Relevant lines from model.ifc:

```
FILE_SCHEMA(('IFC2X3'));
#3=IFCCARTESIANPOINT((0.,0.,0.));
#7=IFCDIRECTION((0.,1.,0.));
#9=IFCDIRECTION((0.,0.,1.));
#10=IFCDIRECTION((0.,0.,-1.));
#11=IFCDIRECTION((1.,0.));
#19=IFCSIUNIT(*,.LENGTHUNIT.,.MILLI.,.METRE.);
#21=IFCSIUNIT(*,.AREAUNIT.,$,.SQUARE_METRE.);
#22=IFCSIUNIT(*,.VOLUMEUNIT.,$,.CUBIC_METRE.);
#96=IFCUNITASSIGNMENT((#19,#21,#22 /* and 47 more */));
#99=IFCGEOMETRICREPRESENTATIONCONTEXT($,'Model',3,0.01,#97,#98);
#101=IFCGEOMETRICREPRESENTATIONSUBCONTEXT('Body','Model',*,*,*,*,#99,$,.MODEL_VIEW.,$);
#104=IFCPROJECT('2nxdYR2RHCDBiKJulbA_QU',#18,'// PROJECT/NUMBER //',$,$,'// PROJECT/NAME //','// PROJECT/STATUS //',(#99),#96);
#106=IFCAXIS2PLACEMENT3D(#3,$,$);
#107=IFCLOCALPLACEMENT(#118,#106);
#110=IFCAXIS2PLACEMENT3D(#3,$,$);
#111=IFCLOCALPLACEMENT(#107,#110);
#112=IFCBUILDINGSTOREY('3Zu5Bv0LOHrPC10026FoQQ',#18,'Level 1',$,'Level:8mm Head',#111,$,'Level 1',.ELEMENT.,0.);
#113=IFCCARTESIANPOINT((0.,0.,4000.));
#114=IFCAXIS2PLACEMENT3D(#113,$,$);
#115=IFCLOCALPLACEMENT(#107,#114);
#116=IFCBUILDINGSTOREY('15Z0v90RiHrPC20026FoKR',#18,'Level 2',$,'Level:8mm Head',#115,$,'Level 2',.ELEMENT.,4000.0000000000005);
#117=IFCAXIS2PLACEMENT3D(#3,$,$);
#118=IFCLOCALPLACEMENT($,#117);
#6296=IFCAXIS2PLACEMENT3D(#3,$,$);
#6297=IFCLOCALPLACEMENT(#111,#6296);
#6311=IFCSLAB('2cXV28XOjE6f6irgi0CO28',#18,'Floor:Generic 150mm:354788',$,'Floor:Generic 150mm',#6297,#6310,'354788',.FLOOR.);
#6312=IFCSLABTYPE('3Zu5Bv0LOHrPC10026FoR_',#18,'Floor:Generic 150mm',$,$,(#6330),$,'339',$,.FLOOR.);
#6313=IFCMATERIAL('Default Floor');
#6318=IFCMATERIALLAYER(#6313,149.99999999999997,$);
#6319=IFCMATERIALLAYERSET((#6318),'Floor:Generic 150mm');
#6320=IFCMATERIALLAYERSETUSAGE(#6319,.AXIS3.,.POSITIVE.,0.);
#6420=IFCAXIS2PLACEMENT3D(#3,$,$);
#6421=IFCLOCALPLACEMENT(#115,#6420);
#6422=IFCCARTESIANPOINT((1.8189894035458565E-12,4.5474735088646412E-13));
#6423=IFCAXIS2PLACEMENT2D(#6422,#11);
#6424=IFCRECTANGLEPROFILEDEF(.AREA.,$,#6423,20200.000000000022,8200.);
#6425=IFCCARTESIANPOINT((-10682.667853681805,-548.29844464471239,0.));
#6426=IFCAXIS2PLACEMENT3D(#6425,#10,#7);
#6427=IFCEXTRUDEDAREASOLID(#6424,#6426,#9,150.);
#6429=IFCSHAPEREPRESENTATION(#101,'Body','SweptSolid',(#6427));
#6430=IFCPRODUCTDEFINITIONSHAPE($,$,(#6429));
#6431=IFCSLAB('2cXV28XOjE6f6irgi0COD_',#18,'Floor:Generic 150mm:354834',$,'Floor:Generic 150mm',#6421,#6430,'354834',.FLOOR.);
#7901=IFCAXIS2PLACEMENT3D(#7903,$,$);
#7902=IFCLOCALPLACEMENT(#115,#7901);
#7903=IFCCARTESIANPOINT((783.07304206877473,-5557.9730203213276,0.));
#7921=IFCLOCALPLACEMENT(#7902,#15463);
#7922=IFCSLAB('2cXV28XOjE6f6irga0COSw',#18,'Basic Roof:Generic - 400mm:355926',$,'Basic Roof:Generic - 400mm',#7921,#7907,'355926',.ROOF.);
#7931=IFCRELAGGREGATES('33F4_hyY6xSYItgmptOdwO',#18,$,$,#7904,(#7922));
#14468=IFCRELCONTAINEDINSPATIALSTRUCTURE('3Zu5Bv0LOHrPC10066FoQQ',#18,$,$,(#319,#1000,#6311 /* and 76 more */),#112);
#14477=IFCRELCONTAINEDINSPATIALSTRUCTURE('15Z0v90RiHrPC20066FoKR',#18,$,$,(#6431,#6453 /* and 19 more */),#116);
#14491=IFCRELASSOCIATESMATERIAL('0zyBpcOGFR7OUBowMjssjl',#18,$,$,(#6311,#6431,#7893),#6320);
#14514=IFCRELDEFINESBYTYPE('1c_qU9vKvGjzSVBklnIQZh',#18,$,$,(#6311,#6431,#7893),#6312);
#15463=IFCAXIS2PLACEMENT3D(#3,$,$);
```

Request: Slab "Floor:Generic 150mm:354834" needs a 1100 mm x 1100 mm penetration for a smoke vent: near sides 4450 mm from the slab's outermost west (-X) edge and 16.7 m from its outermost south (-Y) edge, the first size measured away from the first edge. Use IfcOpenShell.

```python
import numpy as np
import ifcopenshell
import ifcopenshell.api.feature
import ifcopenshell.api.geometry
import ifcopenshell.api.root
import ifcopenshell.geom
import ifcopenshell.util.placement
import ifcopenshell.util.representation
import ifcopenshell.util.shape
import ifcopenshell.util.unit

model = ifcopenshell.open("model.ifc")
unit_scale = ifcopenshell.util.unit.calculate_unit_scale(model)
settings = ifcopenshell.geom.settings()


def volume(element):
    """Net volume in cubic metres, openings subtracted."""
    shape = ifcopenshell.geom.create_shape(settings, element)
    return ifcopenshell.util.shape.get_volume(shape.geometry)


slab = model.by_id(6431)
before = volume(slab)

# Extent in the slab's own axes, in metres. The edges named are its -X and -Y sides.
slab_shape = ifcopenshell.geom.create_shape(settings, slab)
vertices = ifcopenshell.util.shape.get_vertices(slab_shape.geometry)
x_min, y_min, bottom = vertices.min(axis=0)
top = vertices[:, 2].max()

opening = ifcopenshell.api.root.create_entity(model, ifc_class="IfcOpeningElement", name="Smoke vent opening")
context = ifcopenshell.util.representation.get_context(model, "Model", "Body", "MODEL_VIEW")
width, depth = 1.1, 1.1
outline = [(0.0, 0.0), (width, 0.0), (width, depth), (0.0, depth), (0.0, 0.0)]
# Overshoot both faces by 50 mm so the cut is clean.
shape = ifcopenshell.api.geometry.add_slab_representation(
    model, context=context, depth=top - bottom + 0.1, polyline=outline
)
ifcopenshell.api.geometry.assign_representation(model, product=opening, representation=shape)

matrix = ifcopenshell.util.placement.get_local_placement(slab.ObjectPlacement)
matrix[:, 3] = matrix @ np.append(np.array([x_min + 4.45, y_min + 16.7, bottom - 0.05]) / unit_scale, 1.0)
ifcopenshell.api.geometry.edit_object_placement(model, product=opening, matrix=matrix, is_si=False)
ifcopenshell.api.feature.add_feature(model, feature=opening, element=slab)

after = volume(slab)

print(f"slab volume {before:.3f} -> {after:.3f} m3")

model.write("model_rev.ifc")
```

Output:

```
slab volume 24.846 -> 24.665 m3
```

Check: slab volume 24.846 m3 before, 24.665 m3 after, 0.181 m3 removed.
